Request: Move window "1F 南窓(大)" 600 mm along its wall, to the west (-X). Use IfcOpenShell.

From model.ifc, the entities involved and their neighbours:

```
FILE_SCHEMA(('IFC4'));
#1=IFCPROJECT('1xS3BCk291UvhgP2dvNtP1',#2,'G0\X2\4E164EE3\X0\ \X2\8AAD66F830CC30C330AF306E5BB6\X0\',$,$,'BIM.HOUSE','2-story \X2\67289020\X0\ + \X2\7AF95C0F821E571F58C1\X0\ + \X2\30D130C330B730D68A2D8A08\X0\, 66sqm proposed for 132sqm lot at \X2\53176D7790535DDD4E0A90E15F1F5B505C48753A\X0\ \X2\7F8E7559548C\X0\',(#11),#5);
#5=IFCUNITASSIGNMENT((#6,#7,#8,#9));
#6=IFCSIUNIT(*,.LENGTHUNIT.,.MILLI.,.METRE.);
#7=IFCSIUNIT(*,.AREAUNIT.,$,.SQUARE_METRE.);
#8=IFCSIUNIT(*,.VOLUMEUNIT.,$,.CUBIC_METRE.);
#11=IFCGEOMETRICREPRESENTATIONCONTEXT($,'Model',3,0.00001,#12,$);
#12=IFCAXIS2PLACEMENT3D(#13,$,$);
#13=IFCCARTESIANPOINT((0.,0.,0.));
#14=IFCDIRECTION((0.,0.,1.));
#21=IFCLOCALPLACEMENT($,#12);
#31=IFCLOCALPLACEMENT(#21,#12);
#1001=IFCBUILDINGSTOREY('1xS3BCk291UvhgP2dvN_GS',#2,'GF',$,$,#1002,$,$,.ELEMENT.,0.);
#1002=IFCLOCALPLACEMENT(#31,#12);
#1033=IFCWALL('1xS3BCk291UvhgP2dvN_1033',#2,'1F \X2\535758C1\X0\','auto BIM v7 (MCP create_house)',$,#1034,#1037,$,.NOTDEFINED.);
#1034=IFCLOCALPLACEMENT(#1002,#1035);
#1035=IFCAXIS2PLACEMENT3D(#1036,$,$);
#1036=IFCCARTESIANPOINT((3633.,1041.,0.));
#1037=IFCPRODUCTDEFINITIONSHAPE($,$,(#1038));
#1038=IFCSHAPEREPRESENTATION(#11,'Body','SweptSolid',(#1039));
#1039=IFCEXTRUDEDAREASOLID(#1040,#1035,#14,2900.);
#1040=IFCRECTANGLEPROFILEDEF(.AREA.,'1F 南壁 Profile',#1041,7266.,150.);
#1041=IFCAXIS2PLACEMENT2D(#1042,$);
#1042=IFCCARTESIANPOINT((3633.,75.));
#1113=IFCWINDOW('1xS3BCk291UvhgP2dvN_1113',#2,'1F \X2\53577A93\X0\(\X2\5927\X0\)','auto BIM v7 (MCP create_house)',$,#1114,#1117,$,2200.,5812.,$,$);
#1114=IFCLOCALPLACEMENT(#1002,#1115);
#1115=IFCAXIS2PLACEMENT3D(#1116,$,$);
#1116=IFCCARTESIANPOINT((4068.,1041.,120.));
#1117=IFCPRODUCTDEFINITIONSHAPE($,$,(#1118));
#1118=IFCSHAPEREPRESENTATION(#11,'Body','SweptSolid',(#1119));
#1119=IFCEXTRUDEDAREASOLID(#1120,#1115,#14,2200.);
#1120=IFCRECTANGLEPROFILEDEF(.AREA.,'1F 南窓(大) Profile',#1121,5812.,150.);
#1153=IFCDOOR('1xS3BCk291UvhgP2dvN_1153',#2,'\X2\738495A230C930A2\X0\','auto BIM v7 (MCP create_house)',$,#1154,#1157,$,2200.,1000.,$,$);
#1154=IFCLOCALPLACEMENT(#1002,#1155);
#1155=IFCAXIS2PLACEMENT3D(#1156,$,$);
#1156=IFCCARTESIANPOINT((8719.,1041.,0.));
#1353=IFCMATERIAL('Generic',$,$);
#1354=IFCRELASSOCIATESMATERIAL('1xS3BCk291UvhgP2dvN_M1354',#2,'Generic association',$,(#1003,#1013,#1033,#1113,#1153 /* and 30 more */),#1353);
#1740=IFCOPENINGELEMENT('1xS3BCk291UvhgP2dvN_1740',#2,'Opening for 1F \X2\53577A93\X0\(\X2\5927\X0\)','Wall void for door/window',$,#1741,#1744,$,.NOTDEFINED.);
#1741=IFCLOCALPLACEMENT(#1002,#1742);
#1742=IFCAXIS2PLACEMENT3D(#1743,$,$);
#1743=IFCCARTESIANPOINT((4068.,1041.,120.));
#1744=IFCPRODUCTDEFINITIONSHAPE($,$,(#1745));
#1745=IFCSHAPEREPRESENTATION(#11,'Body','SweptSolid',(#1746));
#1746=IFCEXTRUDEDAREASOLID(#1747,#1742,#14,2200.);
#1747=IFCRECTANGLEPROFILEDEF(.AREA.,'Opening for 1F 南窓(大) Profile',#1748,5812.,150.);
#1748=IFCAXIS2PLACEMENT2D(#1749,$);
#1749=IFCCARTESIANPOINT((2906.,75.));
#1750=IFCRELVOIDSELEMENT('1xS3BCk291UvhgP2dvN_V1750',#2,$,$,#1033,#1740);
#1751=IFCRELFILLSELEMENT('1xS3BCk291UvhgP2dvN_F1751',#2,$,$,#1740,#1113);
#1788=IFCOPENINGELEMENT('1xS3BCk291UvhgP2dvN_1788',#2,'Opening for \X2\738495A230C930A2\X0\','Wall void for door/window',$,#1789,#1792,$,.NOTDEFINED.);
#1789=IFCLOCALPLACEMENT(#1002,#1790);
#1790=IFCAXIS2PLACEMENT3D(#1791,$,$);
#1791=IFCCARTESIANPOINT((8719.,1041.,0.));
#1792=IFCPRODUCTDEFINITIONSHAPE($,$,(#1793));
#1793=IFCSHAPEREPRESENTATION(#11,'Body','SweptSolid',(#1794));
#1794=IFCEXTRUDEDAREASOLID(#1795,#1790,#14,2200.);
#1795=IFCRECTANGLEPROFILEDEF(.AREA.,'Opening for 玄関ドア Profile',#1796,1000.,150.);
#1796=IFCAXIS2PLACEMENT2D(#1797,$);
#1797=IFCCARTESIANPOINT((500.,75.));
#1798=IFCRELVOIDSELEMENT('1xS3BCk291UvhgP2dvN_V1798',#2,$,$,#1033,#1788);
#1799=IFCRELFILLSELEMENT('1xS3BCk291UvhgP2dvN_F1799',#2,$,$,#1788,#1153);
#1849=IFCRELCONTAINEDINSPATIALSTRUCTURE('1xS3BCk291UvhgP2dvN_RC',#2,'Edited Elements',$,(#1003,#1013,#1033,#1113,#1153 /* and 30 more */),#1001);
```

```python
import ifcopenshell
import ifcopenshell.api.geometry
import ifcopenshell.util.placement

model = ifcopenshell.open("model.ifc")

window = model.by_id(1113)
opening = window.FillsVoids[0].RelatingOpeningElement
wall = opening.VoidsElements[0].RelatingBuildingElement

wall_matrix = ifcopenshell.util.placement.get_local_placement(wall.ObjectPlacement)
shift = wall_matrix[:3, 0] * -600.0
before = ifcopenshell.util.placement.get_local_placement(window.ObjectPlacement)[:3, 3].copy()

# The window is not placed relative to its opening, so move both.
for product in (opening, window):
    matrix = ifcopenshell.util.placement.get_local_placement(product.ObjectPlacement)
    matrix[:3, 3] += shift
    ifcopenshell.api.geometry.edit_object_placement(model, product=product, matrix=matrix, is_si=False)

after = ifcopenshell.util.placement.get_local_placement(window.ObjectPlacement)[:3, 3]
print("window moved by", (after - before).round(3) + 0.0)

model.write("model-out.ifc")
```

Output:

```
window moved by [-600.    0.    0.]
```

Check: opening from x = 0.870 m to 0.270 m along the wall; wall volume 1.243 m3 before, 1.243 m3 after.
